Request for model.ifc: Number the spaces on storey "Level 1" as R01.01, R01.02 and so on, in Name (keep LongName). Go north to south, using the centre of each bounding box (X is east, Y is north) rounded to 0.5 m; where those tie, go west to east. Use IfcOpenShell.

First a look at what the model holds.

```python
import ifcopenshell
import ifcopenshell.util.element
import ifcopenshell.util.placement

model = ifcopenshell.open("model.ifc")
print(model.schema)
storey = next(s for s in model.by_type("IfcBuildingStorey") if s.Name == "Level 1")
spaces = [e for e in ifcopenshell.util.element.get_decomposition(storey) if e.is_a("IfcSpace")]
for e in sorted(spaces, key=lambda e: e.id()):
    origin = ifcopenshell.util.placement.get_local_placement(e.ObjectPlacement)[:3, 3]
    print(e.id(), e.Name, e.LongName, origin.round(2) + 0.0, sep=" | ")
```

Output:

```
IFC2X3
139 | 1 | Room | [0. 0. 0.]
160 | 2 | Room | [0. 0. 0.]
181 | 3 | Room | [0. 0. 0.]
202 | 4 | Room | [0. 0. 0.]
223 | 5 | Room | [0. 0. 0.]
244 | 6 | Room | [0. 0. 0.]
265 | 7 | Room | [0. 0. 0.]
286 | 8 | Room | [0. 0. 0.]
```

```python
import ifcopenshell
import ifcopenshell.geom
import ifcopenshell.util.element
import ifcopenshell.util.shape

model = ifcopenshell.open("model.ifc")
settings = ifcopenshell.geom.settings()
settings.set("use-world-coords", True)


def centre(element):
    shape = ifcopenshell.geom.create_shape(settings, element)
    return ifcopenshell.util.shape.get_bbox_centroid(shape.geometry)


storey = next(s for s in model.by_type("IfcBuildingStorey") if s.Name == "Level 1")
spaces = [e for e in ifcopenshell.util.element.get_decomposition(storey) if e.is_a("IfcSpace")]

# Insertion points can sit at a corner or the storey origin, so sort by the geometry (in metres).
centres = {e: centre(e) for e in spaces}
spaces.sort(key=lambda e: (-round(centres[e][1] / 0.5), centres[e][0]))

for i, e in enumerate(spaces, start=1):
    number = f"R01.{i:02d}"
    e.Name = number
    print(e.id(), number)

model.write("model-out.ifc")
```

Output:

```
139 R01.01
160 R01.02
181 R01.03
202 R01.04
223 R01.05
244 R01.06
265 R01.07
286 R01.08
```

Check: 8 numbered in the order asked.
